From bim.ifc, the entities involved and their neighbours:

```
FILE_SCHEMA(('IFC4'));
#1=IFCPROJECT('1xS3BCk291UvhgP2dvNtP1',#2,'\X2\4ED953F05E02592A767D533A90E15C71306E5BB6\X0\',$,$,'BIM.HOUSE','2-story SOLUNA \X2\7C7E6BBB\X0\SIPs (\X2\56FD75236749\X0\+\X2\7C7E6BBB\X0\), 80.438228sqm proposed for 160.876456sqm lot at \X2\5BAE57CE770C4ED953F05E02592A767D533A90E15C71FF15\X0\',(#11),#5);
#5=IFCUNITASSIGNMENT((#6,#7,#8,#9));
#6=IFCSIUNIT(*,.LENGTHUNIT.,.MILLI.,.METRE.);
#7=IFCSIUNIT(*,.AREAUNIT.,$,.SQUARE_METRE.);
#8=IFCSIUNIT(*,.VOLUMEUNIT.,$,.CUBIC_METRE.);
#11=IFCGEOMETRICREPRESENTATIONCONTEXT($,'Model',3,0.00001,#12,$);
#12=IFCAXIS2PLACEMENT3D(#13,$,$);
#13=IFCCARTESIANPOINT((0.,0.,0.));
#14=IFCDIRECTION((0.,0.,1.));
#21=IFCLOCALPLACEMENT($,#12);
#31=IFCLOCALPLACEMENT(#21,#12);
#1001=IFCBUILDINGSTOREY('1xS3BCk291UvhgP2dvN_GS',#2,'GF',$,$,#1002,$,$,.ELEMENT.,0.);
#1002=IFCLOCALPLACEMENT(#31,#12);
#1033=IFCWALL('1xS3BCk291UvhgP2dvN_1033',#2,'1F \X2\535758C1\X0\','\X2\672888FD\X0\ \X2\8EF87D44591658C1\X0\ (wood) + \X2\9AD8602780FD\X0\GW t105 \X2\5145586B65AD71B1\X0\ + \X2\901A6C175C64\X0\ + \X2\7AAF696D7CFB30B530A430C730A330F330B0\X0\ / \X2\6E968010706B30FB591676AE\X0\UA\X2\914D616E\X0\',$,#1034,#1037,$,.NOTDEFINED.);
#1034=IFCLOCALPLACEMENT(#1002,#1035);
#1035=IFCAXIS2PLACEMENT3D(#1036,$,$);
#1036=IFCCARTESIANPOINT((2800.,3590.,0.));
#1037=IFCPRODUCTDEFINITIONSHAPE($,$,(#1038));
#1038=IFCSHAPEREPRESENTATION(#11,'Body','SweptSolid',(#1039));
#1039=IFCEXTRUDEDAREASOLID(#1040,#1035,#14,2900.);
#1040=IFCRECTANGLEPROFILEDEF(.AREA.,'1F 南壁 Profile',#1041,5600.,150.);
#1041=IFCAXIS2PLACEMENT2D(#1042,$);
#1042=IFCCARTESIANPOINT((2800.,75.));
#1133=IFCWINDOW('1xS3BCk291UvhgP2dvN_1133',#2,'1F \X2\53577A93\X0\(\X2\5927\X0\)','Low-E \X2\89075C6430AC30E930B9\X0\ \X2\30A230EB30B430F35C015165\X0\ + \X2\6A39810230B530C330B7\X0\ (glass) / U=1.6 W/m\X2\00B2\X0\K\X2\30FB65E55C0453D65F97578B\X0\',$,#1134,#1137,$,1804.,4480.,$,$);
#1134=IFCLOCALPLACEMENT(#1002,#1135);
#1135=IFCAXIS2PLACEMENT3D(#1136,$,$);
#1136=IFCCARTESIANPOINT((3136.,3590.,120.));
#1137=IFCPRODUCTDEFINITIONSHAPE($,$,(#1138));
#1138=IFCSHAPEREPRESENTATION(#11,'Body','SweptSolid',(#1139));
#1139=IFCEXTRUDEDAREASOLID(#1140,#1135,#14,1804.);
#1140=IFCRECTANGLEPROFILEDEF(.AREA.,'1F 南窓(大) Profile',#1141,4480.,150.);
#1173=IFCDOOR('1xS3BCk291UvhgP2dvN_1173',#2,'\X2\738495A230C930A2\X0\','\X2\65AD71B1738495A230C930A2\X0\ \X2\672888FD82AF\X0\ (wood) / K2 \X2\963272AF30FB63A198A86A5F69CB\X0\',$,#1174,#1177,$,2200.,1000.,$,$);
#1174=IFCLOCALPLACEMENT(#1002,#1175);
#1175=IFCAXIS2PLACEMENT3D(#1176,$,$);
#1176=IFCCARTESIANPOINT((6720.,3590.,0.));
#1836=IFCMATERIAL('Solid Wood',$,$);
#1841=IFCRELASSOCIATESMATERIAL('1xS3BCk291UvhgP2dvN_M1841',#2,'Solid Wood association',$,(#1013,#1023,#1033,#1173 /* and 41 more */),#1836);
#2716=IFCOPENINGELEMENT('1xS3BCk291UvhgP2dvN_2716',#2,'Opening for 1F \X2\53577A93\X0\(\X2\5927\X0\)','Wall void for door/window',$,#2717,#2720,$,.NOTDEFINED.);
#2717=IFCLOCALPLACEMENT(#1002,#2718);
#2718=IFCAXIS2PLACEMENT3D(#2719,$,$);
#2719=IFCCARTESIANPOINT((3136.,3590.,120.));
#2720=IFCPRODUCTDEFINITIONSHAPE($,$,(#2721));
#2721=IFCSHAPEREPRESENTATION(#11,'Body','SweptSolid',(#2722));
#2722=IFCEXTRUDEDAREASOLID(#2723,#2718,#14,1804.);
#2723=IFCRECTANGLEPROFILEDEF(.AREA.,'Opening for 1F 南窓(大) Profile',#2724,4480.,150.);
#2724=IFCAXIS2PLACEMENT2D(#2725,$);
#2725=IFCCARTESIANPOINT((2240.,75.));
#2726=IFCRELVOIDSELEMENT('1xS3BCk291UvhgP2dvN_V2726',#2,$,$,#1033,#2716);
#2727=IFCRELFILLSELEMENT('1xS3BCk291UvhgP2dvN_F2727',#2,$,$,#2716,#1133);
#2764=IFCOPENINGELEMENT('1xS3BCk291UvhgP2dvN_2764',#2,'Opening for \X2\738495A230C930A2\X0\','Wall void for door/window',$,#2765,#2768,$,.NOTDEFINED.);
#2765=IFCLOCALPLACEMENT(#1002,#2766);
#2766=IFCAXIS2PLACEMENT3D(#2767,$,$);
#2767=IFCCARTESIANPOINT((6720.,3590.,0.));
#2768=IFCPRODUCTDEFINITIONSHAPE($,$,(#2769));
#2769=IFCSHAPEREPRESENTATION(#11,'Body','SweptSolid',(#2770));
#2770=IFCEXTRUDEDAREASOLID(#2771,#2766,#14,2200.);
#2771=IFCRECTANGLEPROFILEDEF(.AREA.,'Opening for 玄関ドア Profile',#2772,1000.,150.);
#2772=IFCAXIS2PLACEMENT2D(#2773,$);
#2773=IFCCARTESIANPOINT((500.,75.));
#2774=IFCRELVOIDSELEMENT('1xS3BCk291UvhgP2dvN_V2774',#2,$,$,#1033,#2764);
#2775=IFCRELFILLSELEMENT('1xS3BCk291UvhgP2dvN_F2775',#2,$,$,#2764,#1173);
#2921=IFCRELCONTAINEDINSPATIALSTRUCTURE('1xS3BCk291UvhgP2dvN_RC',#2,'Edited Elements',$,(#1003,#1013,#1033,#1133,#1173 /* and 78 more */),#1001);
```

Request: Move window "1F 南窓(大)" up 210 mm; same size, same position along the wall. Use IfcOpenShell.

```python
import numpy as np
import ifcopenshell
import ifcopenshell.api.geometry
import ifcopenshell.util.placement
import ifcopenshell.util.unit

model = ifcopenshell.open("bim.ifc")
unit_scale = ifcopenshell.util.unit.calculate_unit_scale(model)

window = model.by_guid("1xS3BCk291UvhgP2dvN_1133")
opening = window.FillsVoids[0].RelatingOpeningElement
dz = 0.21 / unit_scale

shift = np.array([0.0, 0.0, dz])
# The window is not placed relative to its opening, so move both.
for product in (opening, window):
    matrix = ifcopenshell.util.placement.get_local_placement(product.ObjectPlacement)
    matrix[:3, 3] += shift
    ifcopenshell.api.geometry.edit_object_placement(model, product=product, matrix=matrix, is_si=False)

print(f"moved by {dz * unit_scale:+.3f} m")

model.write("bim-out.ifc")
```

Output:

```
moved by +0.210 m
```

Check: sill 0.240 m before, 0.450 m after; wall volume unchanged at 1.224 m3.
